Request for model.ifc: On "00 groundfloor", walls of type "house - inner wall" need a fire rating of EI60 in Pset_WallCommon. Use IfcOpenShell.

First a look at what the model holds.

```python
import ifcopenshell
import ifcopenshell.util.element

model = ifcopenshell.open("model.ifc")
print(model.schema)
storey = next(s for s in model.by_type("IfcBuildingStorey") if s.Name == "00 groundfloor")
walls = [e for e in ifcopenshell.util.element.get_decomposition(storey) if e.is_a("IfcWall")]
seen = {}
for e in walls:
    element_type = ifcopenshell.util.element.get_type(e)
    key = (element_type.Name if element_type != e and element_type else None, ifcopenshell.util.element.get_pset(e, "Pset_WallCommon", "FireRating"))
    seen[key] = seen.get(key, 0) + 1
for (name, value), count in sorted(seen.items(), key=str):
    print(count, "x", name, "|", value)
```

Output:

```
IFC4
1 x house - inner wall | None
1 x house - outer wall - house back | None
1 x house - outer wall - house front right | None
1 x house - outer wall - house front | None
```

```python
import ifcopenshell
import ifcopenshell.api.pset
import ifcopenshell.util.element

model = ifcopenshell.open("model.ifc")

storey = next(s for s in model.by_type("IfcBuildingStorey") if s.Name == "00 groundfloor")
walls = [e for e in ifcopenshell.util.element.get_decomposition(storey) if e.is_a("IfcWall")]

count = 0
for e in walls:
    element_type = ifcopenshell.util.element.get_type(e)
    if element_type in (None, e) or element_type.Name != "house - inner wall":
        continue
    # add_pset returns the element's existing set when there is one.
    pset = ifcopenshell.api.pset.add_pset(model, product=e, name="Pset_WallCommon")
    ifcopenshell.api.pset.edit_pset(model, pset=pset, properties={"FireRating": "EI60"})
    count += 1

print(count, "walls updated")

model.write("model-out.ifc")
```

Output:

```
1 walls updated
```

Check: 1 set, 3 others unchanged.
